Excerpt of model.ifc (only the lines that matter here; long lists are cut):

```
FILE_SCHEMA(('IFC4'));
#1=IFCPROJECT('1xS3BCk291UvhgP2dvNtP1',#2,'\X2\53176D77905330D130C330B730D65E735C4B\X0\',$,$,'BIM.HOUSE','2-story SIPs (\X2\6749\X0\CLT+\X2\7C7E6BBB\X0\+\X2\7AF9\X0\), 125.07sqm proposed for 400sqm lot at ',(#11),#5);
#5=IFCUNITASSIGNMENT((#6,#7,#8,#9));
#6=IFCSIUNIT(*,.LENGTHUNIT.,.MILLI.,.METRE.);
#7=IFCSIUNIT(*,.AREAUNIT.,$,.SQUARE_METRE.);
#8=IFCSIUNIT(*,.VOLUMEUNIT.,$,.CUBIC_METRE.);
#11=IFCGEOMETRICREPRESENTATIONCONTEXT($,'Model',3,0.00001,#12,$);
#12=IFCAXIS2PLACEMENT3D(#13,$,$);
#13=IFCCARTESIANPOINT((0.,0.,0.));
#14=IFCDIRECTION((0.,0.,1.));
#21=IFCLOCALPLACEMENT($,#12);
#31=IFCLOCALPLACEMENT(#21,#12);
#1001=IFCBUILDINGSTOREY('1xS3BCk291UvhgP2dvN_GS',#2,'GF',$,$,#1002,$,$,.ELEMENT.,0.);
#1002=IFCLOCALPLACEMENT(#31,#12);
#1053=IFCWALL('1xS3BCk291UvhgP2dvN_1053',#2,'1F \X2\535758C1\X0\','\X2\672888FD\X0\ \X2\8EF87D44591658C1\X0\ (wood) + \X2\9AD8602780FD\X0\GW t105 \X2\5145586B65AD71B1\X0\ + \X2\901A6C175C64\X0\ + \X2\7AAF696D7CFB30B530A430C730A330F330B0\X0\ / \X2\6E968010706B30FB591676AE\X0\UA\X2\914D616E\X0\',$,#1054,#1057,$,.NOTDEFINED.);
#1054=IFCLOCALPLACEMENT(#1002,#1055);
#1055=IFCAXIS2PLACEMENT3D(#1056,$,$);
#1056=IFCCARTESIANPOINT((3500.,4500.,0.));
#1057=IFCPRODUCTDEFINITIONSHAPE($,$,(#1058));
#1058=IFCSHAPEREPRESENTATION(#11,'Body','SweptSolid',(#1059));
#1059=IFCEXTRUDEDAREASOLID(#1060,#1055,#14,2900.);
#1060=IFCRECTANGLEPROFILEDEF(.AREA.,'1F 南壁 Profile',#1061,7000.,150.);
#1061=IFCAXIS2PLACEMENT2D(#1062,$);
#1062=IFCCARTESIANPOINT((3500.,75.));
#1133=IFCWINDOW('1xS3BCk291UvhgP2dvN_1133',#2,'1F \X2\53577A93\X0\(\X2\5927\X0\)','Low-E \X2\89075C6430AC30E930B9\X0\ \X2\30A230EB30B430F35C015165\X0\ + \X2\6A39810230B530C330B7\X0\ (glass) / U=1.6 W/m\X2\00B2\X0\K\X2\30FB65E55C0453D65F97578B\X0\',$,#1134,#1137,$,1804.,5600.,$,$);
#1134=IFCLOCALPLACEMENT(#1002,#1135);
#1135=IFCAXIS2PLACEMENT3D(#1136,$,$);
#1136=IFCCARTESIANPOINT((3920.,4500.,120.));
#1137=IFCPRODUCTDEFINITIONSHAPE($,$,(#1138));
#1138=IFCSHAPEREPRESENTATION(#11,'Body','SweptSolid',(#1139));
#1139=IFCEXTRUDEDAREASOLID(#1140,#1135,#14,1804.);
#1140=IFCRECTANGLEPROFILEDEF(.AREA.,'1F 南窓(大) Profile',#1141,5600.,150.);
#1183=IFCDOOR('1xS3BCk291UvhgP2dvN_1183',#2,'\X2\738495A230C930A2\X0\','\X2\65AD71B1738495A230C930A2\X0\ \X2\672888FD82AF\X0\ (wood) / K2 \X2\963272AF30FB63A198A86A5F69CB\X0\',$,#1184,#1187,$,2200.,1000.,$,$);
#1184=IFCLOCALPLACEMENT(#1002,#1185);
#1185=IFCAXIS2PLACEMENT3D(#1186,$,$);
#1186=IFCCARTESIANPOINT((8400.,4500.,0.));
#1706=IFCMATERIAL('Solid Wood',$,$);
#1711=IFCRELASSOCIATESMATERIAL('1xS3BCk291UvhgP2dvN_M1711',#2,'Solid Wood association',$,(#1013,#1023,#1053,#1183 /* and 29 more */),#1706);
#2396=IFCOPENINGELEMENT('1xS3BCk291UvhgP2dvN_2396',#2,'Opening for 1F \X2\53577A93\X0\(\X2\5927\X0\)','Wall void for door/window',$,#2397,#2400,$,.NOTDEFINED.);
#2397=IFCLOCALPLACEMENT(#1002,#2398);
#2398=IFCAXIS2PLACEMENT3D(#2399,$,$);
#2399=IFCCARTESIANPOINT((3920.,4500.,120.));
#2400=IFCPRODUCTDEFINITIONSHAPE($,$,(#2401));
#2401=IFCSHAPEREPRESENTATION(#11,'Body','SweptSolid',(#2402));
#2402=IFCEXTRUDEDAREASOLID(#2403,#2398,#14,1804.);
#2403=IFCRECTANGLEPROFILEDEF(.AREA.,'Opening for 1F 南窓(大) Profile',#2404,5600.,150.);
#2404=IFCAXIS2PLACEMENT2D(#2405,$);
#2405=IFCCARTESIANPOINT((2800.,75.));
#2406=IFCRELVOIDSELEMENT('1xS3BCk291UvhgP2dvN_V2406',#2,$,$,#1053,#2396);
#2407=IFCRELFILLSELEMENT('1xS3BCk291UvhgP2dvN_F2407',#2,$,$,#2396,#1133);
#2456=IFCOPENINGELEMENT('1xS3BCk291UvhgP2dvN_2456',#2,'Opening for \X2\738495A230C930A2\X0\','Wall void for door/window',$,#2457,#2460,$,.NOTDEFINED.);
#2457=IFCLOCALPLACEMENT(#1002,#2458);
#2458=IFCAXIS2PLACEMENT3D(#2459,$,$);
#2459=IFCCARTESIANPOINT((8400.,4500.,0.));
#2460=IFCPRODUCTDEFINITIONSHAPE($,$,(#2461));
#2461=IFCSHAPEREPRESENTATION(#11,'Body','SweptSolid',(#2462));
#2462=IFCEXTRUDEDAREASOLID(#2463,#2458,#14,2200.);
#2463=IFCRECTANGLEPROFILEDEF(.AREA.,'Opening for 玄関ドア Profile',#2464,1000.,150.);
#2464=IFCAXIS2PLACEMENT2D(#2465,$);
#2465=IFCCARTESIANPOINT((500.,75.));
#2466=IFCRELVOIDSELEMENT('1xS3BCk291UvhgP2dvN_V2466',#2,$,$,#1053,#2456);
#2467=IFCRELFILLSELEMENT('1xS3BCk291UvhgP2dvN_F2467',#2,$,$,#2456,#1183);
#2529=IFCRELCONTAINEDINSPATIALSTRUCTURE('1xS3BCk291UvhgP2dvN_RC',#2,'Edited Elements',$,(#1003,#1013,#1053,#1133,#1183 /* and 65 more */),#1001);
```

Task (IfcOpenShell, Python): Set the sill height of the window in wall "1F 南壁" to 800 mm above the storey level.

```python
import numpy as np
import ifcopenshell
import ifcopenshell.api.geometry
import ifcopenshell.geom
import ifcopenshell.util.element
import ifcopenshell.util.placement
import ifcopenshell.util.shape
import ifcopenshell.util.unit

model = ifcopenshell.open("model.ifc")
unit_scale = ifcopenshell.util.unit.calculate_unit_scale(model)

window = model.by_guid("1xS3BCk291UvhgP2dvN_1133")
opening = window.FillsVoids[0].RelatingOpeningElement
storey = ifcopenshell.util.element.get_container(window, ifc_class="IfcBuildingStorey")
level = ifcopenshell.util.placement.get_local_placement(storey.ObjectPlacement)[2, 3]

# The opening's origin need not be at the sill, so measure its lowest point.
shape = ifcopenshell.geom.create_shape(ifcopenshell.geom.settings(), opening)
bottom = ifcopenshell.util.shape.get_shape_bottom_elevation(shape, shape.geometry) / unit_scale
dz = level + 800.0 - bottom

shift = np.array([0.0, 0.0, dz])
# The window is not placed relative to its opening, so move both.
for product in (opening, window):
    matrix = ifcopenshell.util.placement.get_local_placement(product.ObjectPlacement)
    matrix[:3, 3] += shift
    ifcopenshell.api.geometry.edit_object_placement(model, product=product, matrix=matrix, is_si=False)

print(f"moved by {dz * unit_scale:+.3f} m")

model.write("model_v2.ifc")
```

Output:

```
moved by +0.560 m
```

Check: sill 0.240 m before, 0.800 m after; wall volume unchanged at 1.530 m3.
